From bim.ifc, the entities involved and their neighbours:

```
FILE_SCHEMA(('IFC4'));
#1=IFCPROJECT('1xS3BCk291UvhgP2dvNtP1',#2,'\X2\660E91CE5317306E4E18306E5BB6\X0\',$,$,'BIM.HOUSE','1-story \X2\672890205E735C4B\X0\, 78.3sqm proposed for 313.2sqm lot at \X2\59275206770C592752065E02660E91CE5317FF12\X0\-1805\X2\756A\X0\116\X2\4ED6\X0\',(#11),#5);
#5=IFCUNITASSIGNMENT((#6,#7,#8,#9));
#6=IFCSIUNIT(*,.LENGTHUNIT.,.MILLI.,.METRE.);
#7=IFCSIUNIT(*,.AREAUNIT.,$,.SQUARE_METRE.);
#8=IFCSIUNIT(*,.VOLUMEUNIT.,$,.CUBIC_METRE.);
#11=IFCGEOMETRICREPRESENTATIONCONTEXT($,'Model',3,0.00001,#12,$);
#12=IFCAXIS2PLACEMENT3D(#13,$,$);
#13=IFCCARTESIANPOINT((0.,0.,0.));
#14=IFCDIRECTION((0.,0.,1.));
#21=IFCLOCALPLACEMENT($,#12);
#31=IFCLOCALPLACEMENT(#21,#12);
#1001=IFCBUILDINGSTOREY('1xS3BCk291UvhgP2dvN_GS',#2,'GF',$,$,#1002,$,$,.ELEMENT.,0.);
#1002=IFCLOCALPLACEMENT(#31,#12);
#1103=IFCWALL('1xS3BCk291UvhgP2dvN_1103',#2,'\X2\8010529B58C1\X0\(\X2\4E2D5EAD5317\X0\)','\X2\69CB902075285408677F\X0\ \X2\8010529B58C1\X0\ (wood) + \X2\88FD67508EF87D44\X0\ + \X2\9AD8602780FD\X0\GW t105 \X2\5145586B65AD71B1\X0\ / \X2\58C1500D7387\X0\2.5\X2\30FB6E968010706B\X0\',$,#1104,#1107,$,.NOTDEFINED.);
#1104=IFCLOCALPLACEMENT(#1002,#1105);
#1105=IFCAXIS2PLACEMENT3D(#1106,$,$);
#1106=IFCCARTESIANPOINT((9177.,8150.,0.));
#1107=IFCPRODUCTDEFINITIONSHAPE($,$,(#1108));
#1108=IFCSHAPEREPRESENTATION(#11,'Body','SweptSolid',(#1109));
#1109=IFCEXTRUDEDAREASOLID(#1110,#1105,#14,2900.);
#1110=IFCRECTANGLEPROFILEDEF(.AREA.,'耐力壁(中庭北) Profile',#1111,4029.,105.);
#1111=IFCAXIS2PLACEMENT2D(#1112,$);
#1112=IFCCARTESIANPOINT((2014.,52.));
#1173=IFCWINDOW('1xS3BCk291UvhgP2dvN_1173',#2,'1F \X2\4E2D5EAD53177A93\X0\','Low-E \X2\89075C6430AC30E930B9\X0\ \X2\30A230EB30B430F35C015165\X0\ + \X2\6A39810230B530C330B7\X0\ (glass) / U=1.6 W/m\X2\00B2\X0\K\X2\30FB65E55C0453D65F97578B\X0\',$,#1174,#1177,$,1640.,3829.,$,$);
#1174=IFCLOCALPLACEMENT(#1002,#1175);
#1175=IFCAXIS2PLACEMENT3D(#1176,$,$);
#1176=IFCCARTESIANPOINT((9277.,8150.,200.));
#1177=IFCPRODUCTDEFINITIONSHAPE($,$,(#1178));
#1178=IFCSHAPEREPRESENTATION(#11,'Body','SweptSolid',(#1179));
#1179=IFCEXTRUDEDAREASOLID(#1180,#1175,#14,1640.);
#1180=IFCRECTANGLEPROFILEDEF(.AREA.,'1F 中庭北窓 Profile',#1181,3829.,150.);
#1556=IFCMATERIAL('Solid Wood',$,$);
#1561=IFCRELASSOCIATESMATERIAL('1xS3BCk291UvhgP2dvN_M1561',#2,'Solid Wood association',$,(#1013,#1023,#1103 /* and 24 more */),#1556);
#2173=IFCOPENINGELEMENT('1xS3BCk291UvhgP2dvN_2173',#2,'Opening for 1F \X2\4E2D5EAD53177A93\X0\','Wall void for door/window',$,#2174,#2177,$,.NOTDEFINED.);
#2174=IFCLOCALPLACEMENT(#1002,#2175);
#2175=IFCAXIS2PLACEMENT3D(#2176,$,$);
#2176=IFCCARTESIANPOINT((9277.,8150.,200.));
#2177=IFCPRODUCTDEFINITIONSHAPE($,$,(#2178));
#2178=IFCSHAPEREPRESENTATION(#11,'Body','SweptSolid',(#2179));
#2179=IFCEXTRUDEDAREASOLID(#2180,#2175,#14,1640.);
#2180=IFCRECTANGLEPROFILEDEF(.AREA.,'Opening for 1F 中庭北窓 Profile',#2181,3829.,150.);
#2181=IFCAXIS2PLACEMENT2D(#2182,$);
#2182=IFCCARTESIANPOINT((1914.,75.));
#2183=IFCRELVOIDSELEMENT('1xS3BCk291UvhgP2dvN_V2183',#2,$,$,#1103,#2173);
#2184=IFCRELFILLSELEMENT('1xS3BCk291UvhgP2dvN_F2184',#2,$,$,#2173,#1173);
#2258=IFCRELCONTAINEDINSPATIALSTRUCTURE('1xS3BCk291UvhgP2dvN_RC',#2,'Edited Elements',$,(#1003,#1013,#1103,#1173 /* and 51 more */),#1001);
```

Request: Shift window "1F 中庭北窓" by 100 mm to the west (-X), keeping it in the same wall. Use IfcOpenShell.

```python
import ifcopenshell
import ifcopenshell.api.geometry
import ifcopenshell.util.placement

model = ifcopenshell.open("bim.ifc")

window = model.by_id(1173)
opening = window.FillsVoids[0].RelatingOpeningElement
wall = opening.VoidsElements[0].RelatingBuildingElement

wall_matrix = ifcopenshell.util.placement.get_local_placement(wall.ObjectPlacement)
shift = wall_matrix[:3, 0] * -100.0
before = ifcopenshell.util.placement.get_local_placement(window.ObjectPlacement)[:3, 3].copy()

# The window is not placed relative to its opening, so move both.
for product in (opening, window):
    matrix = ifcopenshell.util.placement.get_local_placement(product.ObjectPlacement)
    matrix[:3, 3] += shift
    ifcopenshell.api.geometry.edit_object_placement(model, product=product, matrix=matrix, is_si=False)

after = ifcopenshell.util.placement.get_local_placement(window.ObjectPlacement)[:3, 3]
print("window moved by", (after - before).round(3) + 0.0)

model.write("bim_edited.ifc")
```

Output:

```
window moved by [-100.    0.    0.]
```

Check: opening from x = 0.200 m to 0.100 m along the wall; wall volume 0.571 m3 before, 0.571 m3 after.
